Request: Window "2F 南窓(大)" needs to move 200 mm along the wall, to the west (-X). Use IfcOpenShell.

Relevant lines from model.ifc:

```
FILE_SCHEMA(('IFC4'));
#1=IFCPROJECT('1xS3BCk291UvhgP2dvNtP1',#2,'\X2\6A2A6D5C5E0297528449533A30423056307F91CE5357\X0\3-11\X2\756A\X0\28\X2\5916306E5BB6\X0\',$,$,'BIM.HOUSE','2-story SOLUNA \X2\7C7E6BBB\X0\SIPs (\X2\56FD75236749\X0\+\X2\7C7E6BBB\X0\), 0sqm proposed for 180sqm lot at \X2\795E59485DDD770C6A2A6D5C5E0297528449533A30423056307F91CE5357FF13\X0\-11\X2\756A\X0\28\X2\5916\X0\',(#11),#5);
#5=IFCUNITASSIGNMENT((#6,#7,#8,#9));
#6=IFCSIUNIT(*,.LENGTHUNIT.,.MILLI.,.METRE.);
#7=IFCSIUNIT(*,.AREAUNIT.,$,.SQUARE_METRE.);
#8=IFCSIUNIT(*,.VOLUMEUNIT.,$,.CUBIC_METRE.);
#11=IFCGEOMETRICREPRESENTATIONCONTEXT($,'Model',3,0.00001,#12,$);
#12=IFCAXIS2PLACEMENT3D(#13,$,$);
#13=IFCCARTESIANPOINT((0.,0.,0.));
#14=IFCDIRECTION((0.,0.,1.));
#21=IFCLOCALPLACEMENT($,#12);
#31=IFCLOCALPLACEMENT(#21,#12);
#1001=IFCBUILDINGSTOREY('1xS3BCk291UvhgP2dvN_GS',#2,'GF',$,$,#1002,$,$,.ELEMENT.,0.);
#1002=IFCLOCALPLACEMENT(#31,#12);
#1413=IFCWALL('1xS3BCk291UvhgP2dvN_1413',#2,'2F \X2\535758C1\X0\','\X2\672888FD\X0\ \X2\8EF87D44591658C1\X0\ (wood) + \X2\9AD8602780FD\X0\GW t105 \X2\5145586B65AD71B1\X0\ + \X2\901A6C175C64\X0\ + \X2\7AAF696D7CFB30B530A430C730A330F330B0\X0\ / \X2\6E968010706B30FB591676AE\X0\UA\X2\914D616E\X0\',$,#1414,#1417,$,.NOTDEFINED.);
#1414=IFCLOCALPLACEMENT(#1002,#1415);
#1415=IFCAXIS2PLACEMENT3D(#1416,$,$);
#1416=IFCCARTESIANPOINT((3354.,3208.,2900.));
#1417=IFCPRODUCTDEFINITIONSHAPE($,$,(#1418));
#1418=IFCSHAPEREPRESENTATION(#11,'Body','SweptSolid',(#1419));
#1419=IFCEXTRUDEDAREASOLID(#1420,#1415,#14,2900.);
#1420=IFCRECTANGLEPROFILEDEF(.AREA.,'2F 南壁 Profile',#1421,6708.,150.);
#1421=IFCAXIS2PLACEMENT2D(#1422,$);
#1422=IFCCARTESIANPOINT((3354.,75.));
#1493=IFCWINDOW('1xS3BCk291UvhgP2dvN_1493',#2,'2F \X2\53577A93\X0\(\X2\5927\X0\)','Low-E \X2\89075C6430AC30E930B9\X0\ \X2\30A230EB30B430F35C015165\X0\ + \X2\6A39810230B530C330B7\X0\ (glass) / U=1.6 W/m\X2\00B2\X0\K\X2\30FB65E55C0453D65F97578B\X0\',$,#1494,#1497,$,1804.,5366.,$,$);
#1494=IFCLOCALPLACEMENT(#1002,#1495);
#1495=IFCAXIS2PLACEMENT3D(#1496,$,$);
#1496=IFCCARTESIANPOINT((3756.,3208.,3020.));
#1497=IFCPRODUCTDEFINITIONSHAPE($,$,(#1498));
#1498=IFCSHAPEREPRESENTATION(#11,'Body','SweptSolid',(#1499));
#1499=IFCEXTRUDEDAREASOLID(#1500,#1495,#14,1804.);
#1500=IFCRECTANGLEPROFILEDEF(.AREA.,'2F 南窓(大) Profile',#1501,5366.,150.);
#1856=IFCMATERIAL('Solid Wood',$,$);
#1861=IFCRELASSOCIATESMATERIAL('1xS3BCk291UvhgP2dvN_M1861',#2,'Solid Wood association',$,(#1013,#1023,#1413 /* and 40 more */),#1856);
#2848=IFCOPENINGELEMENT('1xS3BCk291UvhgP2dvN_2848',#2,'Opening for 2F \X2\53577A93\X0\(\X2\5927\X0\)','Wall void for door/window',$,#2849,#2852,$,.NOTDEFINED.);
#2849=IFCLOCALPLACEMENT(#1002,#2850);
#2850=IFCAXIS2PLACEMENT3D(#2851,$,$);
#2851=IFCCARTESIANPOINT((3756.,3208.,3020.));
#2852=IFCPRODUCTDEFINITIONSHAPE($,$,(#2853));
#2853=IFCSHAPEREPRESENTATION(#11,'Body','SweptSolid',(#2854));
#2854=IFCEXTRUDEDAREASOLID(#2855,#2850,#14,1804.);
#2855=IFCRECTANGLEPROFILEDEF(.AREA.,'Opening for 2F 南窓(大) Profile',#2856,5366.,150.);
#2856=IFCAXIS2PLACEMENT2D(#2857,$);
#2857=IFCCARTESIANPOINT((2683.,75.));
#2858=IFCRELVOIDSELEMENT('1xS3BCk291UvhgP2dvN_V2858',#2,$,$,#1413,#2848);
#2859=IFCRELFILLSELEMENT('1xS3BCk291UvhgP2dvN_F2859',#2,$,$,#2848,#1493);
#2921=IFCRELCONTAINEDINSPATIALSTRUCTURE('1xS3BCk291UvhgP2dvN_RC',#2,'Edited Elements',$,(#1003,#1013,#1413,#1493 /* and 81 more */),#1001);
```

```python
import ifcopenshell
import ifcopenshell.api.geometry
import ifcopenshell.util.placement
import ifcopenshell.util.unit

model = ifcopenshell.open("model.ifc")
unit_scale = ifcopenshell.util.unit.calculate_unit_scale(model)

window = model.by_guid("1xS3BCk291UvhgP2dvN_1493")
opening = window.FillsVoids[0].RelatingOpeningElement
wall = opening.VoidsElements[0].RelatingBuildingElement

wall_matrix = ifcopenshell.util.placement.get_local_placement(wall.ObjectPlacement)
shift = wall_matrix[:3, 0] * -0.2 / unit_scale
before = ifcopenshell.util.placement.get_local_placement(window.ObjectPlacement)[:3, 3].copy()

# The window is not placed relative to its opening, so move both.
for product in (opening, window):
    matrix = ifcopenshell.util.placement.get_local_placement(product.ObjectPlacement)
    matrix[:3, 3] += shift
    ifcopenshell.api.geometry.edit_object_placement(model, product=product, matrix=matrix, is_si=False)

after = ifcopenshell.util.placement.get_local_placement(window.ObjectPlacement)[:3, 3]
print("window moved by", (after - before).round(3) + 0.0)

model.write("model_rev.ifc")
```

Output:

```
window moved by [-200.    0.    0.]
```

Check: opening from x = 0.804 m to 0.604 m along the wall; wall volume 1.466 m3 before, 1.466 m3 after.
